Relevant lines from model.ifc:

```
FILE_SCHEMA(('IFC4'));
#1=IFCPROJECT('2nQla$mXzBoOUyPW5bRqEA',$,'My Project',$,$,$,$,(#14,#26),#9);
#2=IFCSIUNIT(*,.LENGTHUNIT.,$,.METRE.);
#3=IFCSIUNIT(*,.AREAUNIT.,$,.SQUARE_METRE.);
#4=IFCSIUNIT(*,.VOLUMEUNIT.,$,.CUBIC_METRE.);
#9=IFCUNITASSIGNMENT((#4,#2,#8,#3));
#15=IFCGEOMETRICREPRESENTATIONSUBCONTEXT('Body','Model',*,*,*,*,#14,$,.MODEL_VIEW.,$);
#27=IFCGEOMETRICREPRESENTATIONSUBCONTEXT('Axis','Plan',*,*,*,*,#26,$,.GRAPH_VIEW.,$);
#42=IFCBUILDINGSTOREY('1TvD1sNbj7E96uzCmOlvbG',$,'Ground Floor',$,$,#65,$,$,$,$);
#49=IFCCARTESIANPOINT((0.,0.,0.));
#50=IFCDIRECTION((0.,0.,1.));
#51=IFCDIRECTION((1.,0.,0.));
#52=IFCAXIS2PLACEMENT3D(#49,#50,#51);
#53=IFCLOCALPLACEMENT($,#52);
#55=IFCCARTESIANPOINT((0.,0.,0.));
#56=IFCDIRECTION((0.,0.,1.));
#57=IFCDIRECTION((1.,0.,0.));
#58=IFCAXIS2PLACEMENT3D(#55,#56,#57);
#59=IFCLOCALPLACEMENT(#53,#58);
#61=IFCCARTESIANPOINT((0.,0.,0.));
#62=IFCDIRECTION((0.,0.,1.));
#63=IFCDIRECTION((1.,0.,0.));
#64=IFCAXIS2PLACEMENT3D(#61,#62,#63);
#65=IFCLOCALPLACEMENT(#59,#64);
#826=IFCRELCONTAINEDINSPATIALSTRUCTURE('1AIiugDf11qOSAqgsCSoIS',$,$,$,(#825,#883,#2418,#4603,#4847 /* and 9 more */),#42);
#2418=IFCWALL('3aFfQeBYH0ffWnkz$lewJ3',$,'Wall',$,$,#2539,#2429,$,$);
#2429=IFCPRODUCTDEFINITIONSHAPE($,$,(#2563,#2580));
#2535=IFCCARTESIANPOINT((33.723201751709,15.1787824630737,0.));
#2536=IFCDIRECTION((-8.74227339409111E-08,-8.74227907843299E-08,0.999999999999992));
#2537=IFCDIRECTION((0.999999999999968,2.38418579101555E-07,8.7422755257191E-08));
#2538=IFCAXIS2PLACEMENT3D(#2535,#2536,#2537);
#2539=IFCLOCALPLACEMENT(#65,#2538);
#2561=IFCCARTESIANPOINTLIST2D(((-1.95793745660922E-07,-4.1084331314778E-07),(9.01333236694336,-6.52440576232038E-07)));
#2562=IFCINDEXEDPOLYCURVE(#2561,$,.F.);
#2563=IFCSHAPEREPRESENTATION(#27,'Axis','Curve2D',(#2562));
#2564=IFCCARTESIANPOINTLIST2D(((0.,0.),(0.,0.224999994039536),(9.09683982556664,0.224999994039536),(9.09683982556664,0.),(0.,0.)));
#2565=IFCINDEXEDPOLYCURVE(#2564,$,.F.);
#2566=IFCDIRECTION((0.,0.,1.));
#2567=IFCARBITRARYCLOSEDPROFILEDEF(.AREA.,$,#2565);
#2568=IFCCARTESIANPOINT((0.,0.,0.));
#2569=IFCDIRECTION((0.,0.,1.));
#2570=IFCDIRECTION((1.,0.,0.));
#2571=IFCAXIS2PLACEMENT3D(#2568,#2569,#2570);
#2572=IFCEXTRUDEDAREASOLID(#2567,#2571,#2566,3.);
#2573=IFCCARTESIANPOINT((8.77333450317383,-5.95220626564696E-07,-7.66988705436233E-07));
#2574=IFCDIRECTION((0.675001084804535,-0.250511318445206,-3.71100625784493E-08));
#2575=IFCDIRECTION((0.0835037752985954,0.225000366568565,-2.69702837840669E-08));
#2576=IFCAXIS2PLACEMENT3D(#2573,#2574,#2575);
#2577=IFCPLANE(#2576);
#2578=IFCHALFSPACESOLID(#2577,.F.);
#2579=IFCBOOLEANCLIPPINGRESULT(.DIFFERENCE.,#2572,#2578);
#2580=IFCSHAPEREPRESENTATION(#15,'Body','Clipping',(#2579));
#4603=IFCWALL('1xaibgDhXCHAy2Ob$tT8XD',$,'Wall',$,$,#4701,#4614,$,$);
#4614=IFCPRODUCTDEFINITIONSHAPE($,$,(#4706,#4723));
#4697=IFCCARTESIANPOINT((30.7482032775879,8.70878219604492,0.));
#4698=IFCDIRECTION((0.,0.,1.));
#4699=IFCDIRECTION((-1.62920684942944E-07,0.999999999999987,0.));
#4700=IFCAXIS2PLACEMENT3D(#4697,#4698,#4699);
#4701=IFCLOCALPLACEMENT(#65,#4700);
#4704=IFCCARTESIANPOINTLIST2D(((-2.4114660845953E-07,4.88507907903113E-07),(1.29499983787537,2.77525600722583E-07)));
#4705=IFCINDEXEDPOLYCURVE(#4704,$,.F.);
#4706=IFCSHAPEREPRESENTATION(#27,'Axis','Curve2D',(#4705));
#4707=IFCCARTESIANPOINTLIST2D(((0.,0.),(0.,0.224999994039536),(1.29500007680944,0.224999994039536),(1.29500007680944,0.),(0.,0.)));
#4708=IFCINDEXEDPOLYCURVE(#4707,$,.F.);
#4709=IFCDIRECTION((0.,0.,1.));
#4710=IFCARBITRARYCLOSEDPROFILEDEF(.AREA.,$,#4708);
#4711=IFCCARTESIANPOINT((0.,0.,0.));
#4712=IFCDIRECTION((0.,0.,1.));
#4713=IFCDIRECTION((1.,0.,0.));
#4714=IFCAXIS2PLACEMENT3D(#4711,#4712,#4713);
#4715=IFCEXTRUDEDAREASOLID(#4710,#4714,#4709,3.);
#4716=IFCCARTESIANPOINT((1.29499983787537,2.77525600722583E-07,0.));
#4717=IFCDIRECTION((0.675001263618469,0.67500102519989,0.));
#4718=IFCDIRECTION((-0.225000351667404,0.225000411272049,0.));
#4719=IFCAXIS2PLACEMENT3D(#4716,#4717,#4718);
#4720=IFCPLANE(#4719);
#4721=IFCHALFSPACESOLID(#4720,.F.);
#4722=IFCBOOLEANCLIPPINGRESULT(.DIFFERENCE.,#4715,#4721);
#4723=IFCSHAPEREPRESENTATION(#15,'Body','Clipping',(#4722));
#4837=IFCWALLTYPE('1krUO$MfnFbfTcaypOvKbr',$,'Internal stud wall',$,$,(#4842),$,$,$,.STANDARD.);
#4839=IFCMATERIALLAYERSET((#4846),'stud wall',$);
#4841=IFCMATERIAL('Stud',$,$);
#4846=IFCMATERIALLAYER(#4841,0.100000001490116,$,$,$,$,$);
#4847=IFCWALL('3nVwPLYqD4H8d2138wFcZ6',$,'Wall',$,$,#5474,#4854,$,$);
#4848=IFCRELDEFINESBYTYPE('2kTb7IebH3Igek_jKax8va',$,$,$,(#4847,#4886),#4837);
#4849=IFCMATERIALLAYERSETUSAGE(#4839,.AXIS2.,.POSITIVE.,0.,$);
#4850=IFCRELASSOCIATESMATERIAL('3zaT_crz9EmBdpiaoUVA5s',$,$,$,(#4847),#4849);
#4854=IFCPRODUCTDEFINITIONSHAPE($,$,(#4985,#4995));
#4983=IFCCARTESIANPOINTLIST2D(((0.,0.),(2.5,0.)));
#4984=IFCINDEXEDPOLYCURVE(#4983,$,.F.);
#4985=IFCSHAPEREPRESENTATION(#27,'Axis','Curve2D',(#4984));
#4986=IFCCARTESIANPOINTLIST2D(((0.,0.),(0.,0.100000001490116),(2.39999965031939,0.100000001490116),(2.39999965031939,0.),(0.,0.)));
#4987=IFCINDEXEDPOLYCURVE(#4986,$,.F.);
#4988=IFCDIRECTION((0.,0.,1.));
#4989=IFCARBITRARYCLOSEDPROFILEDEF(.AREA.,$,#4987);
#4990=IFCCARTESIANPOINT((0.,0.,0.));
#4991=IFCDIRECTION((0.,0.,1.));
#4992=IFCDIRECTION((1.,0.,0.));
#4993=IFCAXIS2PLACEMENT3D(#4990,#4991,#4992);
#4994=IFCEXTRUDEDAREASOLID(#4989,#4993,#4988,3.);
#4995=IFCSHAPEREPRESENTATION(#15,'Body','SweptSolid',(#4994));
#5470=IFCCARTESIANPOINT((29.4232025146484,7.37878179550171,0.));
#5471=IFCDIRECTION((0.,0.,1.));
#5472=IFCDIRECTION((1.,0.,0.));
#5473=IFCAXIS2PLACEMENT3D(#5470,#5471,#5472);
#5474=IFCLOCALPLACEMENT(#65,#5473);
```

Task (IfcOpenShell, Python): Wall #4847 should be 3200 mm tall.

```python
import ifcopenshell
import ifcopenshell.geom
import ifcopenshell.util.representation
import ifcopenshell.util.shape
import ifcopenshell.util.unit

model = ifcopenshell.open("model.ifc")
unit_scale = ifcopenshell.util.unit.calculate_unit_scale(model)
settings = ifcopenshell.geom.settings()


def volume(element):
    """Net volume in cubic metres, openings subtracted."""
    shape = ifcopenshell.geom.create_shape(settings, element)
    return ifcopenshell.util.shape.get_volume(shape.geometry)


wall = model.by_guid("3nVwPLYqD4H8d2138wFcZ6")
before = volume(wall)

body = ifcopenshell.util.representation.get_representation(wall, "Model", "Body")
solid = body.Items[0]
old_height = solid.Depth
solid.Depth = 3.2 / unit_scale
after = volume(wall)

print(f"height {old_height:g} -> {solid.Depth:g}, volume {before:.3f} -> {after:.3f} m3")

model.write("model_edited.ifc")
```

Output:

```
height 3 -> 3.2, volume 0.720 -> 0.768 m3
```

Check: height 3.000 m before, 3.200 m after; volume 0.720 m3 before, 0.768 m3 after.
